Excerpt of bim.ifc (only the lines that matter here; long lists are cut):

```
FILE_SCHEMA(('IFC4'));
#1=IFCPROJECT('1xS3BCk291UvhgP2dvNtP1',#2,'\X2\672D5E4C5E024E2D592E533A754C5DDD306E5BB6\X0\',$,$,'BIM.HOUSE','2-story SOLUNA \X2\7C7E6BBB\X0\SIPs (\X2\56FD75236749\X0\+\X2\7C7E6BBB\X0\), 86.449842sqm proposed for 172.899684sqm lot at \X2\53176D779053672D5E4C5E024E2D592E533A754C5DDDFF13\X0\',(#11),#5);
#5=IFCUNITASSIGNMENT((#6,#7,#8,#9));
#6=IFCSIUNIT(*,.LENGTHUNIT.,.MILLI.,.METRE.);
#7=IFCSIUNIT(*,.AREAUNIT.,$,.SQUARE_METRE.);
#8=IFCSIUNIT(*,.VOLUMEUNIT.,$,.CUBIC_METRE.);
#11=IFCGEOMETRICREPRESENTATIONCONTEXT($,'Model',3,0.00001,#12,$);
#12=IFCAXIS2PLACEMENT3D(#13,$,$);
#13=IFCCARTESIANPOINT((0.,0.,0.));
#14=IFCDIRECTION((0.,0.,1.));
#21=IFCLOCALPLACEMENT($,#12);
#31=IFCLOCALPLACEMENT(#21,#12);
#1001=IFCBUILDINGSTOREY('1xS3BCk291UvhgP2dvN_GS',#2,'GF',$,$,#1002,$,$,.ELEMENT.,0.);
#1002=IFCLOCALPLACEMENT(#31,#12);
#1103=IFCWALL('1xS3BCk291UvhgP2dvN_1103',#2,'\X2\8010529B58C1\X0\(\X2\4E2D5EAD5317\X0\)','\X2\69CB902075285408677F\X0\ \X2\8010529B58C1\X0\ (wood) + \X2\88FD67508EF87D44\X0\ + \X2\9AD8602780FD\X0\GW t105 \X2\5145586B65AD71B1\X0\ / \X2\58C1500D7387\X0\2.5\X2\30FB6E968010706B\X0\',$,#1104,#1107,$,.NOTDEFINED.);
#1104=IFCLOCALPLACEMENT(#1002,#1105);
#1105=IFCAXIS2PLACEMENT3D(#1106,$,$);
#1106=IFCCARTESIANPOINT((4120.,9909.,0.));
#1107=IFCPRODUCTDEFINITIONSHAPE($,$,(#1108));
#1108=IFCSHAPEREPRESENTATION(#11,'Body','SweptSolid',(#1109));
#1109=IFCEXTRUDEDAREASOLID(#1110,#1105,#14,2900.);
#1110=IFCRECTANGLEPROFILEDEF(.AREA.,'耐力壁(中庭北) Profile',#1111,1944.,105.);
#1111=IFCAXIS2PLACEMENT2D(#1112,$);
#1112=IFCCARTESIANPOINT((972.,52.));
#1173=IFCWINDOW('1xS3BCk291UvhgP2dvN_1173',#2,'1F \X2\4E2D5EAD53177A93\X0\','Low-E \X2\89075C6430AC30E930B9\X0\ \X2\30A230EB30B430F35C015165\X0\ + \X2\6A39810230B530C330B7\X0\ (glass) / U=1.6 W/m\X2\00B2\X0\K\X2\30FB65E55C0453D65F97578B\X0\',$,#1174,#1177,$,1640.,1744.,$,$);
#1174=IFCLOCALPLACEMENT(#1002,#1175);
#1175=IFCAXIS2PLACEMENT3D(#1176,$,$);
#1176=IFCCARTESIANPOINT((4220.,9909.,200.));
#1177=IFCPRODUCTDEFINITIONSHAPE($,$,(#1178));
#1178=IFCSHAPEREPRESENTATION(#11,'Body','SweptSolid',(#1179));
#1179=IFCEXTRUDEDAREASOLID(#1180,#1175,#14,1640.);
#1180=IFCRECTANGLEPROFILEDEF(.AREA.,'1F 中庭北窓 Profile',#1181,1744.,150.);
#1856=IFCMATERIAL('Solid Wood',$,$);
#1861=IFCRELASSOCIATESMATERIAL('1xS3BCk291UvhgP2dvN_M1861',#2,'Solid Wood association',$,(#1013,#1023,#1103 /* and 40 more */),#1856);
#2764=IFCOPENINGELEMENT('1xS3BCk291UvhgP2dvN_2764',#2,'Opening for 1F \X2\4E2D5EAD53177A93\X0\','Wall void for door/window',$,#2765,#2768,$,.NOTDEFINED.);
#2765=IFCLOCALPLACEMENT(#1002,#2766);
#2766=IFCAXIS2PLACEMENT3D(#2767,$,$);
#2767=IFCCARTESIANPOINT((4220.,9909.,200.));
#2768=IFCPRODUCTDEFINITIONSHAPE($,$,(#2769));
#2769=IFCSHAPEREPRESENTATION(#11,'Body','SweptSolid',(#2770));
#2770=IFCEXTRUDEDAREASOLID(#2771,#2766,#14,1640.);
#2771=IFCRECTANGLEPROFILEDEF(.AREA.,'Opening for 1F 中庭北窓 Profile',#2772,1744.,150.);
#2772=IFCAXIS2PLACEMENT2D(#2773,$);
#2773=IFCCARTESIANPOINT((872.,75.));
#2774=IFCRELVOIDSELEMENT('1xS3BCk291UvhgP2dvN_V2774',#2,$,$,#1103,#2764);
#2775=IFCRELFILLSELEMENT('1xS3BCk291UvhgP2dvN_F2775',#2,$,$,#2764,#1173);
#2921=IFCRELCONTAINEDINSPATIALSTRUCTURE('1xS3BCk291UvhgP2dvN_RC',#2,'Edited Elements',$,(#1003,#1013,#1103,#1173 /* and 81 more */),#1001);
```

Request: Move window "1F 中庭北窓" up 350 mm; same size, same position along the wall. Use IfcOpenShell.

```python
import numpy as np
import ifcopenshell
import ifcopenshell.api.geometry
import ifcopenshell.util.placement
import ifcopenshell.util.unit

model = ifcopenshell.open("bim.ifc")
unit_scale = ifcopenshell.util.unit.calculate_unit_scale(model)

window = model.by_guid("1xS3BCk291UvhgP2dvN_1173")
opening = window.FillsVoids[0].RelatingOpeningElement
dz = 0.35 / unit_scale

shift = np.array([0.0, 0.0, dz])
# The window is not placed relative to its opening, so move both.
for product in (opening, window):
    matrix = ifcopenshell.util.placement.get_local_placement(product.ObjectPlacement)
    matrix[:3, 3] += shift
    ifcopenshell.api.geometry.edit_object_placement(model, product=product, matrix=matrix, is_si=False)

print(f"moved by {dz * unit_scale:+.3f} m")

model.write("bim-out.ifc")
```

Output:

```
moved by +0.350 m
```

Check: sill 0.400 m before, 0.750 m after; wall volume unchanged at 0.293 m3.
